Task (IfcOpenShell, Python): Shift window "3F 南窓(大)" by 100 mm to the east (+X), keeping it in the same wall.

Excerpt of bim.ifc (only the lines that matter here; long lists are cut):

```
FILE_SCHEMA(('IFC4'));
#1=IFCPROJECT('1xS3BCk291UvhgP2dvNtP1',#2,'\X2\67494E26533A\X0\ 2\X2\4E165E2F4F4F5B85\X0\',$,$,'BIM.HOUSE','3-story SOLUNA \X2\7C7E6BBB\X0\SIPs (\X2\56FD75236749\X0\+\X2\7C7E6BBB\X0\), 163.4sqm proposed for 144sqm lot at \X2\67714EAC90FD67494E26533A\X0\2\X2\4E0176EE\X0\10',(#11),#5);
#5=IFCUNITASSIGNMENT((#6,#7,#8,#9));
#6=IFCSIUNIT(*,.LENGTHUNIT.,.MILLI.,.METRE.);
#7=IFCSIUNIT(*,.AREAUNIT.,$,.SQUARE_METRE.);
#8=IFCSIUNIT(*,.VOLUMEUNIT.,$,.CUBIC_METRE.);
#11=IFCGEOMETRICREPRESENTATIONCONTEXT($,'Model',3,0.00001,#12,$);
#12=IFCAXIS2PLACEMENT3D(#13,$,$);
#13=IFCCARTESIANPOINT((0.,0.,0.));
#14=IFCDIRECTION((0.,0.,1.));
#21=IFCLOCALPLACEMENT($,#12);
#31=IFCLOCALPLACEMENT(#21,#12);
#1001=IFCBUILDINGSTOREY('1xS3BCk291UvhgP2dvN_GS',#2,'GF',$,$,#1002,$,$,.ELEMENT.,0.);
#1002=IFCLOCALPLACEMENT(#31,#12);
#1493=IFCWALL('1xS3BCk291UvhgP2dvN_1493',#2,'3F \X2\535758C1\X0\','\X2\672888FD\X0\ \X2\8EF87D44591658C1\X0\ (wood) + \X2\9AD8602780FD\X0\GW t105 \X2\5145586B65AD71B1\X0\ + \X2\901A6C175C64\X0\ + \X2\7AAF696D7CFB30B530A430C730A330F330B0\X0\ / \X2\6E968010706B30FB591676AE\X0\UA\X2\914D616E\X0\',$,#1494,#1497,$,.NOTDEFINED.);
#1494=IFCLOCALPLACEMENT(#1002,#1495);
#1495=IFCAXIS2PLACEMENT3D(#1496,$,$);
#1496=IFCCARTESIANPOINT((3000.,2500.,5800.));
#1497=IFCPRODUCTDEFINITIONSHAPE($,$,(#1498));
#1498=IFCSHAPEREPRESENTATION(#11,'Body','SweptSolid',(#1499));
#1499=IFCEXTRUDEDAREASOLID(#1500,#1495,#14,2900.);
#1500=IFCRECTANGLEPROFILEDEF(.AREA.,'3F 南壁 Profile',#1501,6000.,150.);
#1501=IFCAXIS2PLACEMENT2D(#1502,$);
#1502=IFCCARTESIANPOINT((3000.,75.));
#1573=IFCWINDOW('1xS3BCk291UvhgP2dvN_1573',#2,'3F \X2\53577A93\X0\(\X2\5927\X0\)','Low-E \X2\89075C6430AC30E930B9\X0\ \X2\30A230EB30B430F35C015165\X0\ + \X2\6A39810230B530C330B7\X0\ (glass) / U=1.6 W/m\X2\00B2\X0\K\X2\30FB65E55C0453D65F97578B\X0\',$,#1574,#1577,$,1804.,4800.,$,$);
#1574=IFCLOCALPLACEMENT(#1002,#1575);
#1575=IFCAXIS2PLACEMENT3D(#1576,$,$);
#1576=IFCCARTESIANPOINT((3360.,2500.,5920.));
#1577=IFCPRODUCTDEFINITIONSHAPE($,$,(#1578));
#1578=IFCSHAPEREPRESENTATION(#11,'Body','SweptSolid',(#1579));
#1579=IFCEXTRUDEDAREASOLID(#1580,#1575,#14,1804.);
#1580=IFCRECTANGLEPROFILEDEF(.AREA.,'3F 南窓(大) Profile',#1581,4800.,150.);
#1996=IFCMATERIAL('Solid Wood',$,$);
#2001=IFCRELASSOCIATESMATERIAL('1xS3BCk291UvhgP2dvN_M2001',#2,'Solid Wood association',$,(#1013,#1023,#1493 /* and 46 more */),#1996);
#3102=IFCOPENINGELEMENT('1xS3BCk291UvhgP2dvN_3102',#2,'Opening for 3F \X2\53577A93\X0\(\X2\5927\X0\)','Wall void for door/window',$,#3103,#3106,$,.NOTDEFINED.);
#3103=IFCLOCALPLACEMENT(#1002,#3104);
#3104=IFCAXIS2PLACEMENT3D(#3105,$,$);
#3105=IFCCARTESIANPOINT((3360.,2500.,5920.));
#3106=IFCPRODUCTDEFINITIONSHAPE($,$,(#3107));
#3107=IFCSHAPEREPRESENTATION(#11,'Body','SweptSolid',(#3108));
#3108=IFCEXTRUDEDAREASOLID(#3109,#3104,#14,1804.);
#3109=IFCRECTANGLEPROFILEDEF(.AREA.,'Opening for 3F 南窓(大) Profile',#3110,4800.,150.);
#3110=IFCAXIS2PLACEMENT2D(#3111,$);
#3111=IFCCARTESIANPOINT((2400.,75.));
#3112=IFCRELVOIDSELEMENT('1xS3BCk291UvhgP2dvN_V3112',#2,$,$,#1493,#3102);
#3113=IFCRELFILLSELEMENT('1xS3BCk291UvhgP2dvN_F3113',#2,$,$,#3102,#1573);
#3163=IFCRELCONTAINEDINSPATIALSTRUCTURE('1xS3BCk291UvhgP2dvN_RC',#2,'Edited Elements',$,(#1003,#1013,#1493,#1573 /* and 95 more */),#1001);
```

```python
import ifcopenshell
import ifcopenshell.api.geometry
import ifcopenshell.util.placement

model = ifcopenshell.open("bim.ifc")

window = model.by_guid("1xS3BCk291UvhgP2dvN_1573")
opening = window.FillsVoids[0].RelatingOpeningElement
wall = opening.VoidsElements[0].RelatingBuildingElement

wall_matrix = ifcopenshell.util.placement.get_local_placement(wall.ObjectPlacement)
shift = wall_matrix[:3, 0] * 100.0
before = ifcopenshell.util.placement.get_local_placement(window.ObjectPlacement)[:3, 3].copy()

# The window is not placed relative to its opening, so move both.
for product in (opening, window):
    matrix = ifcopenshell.util.placement.get_local_placement(product.ObjectPlacement)
    matrix[:3, 3] += shift
    ifcopenshell.api.geometry.edit_object_placement(model, product=product, matrix=matrix, is_si=False)

after = ifcopenshell.util.placement.get_local_placement(window.ObjectPlacement)[:3, 3]
print("window moved by", (after - before).round(3) + 0.0)

model.write("bim_rev.ifc")
```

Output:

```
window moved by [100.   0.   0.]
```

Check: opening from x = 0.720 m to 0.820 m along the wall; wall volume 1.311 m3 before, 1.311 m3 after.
